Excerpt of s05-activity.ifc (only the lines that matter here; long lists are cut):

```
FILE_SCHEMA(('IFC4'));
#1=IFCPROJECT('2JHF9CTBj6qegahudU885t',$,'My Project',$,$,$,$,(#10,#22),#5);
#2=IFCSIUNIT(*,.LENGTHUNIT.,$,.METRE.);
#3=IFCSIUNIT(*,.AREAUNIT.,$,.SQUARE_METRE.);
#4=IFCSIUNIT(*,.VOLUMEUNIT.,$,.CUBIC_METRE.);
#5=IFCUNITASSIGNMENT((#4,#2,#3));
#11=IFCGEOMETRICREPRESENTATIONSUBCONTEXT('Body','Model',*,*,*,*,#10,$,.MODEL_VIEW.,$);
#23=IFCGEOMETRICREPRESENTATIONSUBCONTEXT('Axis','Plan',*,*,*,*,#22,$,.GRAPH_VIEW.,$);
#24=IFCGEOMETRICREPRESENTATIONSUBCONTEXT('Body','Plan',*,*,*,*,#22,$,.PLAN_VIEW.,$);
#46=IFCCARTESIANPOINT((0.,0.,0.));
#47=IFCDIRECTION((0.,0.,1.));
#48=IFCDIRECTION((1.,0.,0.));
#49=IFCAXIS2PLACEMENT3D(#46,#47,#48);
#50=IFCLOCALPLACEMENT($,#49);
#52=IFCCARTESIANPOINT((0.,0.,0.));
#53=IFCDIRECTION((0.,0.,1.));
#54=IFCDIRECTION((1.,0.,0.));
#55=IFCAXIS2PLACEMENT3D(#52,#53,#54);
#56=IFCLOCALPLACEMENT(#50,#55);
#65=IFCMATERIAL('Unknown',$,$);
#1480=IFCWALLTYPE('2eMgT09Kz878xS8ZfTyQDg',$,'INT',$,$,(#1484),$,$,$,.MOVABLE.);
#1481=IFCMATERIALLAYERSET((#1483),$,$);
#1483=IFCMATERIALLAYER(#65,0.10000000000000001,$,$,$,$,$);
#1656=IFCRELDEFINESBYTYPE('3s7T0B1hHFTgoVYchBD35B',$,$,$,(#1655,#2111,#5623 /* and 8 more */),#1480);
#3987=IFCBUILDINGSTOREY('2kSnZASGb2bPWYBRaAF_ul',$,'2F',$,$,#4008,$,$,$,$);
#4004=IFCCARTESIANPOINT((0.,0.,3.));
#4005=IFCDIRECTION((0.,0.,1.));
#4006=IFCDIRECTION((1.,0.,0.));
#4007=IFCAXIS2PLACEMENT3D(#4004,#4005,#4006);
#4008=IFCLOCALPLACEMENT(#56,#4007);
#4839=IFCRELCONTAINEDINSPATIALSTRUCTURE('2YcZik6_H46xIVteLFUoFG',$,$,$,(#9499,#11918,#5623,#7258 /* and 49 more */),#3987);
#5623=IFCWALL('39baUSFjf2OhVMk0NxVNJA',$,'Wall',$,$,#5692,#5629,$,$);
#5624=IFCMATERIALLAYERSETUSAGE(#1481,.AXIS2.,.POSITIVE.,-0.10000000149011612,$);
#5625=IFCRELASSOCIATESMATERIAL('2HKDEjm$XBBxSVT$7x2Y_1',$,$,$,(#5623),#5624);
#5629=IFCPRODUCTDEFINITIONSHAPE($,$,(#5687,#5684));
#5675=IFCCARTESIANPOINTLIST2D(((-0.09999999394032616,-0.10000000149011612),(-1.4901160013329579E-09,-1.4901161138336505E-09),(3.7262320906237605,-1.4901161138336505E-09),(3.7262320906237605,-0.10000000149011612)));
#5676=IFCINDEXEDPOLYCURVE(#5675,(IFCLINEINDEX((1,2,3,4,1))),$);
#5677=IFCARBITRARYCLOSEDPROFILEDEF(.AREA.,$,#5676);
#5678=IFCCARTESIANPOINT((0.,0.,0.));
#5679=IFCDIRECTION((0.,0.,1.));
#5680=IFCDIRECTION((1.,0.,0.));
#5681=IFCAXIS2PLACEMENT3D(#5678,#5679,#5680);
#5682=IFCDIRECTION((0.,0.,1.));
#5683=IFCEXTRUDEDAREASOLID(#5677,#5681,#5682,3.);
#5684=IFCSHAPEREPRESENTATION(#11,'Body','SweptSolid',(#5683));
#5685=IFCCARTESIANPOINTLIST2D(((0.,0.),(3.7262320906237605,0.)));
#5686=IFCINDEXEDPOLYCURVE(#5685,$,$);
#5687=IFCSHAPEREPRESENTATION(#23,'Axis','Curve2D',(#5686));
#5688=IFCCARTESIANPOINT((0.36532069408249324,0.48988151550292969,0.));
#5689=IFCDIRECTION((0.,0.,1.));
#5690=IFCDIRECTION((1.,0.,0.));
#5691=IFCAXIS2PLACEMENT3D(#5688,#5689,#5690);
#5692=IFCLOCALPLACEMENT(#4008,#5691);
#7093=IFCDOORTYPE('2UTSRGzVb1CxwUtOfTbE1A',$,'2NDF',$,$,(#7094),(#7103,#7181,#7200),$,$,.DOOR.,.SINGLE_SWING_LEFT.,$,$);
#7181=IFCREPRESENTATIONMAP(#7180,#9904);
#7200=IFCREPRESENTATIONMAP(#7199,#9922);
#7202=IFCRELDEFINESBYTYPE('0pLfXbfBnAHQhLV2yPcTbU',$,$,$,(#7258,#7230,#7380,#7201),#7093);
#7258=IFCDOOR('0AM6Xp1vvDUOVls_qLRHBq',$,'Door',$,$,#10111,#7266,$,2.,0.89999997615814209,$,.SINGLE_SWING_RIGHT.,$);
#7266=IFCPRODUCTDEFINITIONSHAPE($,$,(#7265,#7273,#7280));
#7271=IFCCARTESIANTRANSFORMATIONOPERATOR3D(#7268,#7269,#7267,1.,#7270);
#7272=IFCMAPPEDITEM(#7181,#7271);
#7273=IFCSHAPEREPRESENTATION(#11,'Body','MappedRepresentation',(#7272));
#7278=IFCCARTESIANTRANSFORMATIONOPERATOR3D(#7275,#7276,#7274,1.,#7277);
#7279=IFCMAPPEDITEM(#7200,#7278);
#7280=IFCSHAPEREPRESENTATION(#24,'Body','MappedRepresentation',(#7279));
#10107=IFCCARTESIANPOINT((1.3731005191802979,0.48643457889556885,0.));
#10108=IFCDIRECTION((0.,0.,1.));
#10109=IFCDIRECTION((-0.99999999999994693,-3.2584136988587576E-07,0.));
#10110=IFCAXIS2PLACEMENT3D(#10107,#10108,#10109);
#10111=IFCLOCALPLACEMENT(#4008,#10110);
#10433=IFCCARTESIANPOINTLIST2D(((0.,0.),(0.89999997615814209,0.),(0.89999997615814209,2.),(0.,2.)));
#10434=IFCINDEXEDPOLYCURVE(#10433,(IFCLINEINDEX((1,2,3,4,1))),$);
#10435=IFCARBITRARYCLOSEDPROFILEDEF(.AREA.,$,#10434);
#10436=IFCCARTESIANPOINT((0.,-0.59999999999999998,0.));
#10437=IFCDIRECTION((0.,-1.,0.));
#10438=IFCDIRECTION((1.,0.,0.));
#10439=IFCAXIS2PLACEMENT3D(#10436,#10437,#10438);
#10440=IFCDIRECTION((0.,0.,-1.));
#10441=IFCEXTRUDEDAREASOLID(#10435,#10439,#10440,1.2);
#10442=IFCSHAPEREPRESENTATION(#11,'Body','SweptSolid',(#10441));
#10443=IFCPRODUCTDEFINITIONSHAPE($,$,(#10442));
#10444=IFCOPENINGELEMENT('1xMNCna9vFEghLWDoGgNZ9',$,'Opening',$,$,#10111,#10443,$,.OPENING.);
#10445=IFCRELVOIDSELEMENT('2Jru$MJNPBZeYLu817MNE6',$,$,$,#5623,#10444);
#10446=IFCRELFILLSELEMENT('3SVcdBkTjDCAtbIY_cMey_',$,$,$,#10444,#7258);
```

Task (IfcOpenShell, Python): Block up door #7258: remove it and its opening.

```python
import ifcopenshell
import ifcopenshell.api.feature
import ifcopenshell.api.root
import ifcopenshell.geom
import ifcopenshell.util.shape

model = ifcopenshell.open("s05-activity.ifc")
settings = ifcopenshell.geom.settings()


def volume(element):
    """Net volume in cubic metres, openings subtracted."""
    shape = ifcopenshell.geom.create_shape(settings, element)
    return ifcopenshell.util.shape.get_volume(shape.geometry)


door = model.by_guid("0AM6Xp1vvDUOVls_qLRHBq")
opening = door.FillsVoids[0].RelatingOpeningElement
wall = opening.VoidsElements[0].RelatingBuildingElement
before = volume(wall)

ifcopenshell.api.root.remove_product(model, product=door)
ifcopenshell.api.feature.remove_feature(model, feature=opening)

after = volume(wall)

print(f"wall volume {before:.3f} -> {after:.3f} m3")

model.write("s05-activity_edited.ifc")
```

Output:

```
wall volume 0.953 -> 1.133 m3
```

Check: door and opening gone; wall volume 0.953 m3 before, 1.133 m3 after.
